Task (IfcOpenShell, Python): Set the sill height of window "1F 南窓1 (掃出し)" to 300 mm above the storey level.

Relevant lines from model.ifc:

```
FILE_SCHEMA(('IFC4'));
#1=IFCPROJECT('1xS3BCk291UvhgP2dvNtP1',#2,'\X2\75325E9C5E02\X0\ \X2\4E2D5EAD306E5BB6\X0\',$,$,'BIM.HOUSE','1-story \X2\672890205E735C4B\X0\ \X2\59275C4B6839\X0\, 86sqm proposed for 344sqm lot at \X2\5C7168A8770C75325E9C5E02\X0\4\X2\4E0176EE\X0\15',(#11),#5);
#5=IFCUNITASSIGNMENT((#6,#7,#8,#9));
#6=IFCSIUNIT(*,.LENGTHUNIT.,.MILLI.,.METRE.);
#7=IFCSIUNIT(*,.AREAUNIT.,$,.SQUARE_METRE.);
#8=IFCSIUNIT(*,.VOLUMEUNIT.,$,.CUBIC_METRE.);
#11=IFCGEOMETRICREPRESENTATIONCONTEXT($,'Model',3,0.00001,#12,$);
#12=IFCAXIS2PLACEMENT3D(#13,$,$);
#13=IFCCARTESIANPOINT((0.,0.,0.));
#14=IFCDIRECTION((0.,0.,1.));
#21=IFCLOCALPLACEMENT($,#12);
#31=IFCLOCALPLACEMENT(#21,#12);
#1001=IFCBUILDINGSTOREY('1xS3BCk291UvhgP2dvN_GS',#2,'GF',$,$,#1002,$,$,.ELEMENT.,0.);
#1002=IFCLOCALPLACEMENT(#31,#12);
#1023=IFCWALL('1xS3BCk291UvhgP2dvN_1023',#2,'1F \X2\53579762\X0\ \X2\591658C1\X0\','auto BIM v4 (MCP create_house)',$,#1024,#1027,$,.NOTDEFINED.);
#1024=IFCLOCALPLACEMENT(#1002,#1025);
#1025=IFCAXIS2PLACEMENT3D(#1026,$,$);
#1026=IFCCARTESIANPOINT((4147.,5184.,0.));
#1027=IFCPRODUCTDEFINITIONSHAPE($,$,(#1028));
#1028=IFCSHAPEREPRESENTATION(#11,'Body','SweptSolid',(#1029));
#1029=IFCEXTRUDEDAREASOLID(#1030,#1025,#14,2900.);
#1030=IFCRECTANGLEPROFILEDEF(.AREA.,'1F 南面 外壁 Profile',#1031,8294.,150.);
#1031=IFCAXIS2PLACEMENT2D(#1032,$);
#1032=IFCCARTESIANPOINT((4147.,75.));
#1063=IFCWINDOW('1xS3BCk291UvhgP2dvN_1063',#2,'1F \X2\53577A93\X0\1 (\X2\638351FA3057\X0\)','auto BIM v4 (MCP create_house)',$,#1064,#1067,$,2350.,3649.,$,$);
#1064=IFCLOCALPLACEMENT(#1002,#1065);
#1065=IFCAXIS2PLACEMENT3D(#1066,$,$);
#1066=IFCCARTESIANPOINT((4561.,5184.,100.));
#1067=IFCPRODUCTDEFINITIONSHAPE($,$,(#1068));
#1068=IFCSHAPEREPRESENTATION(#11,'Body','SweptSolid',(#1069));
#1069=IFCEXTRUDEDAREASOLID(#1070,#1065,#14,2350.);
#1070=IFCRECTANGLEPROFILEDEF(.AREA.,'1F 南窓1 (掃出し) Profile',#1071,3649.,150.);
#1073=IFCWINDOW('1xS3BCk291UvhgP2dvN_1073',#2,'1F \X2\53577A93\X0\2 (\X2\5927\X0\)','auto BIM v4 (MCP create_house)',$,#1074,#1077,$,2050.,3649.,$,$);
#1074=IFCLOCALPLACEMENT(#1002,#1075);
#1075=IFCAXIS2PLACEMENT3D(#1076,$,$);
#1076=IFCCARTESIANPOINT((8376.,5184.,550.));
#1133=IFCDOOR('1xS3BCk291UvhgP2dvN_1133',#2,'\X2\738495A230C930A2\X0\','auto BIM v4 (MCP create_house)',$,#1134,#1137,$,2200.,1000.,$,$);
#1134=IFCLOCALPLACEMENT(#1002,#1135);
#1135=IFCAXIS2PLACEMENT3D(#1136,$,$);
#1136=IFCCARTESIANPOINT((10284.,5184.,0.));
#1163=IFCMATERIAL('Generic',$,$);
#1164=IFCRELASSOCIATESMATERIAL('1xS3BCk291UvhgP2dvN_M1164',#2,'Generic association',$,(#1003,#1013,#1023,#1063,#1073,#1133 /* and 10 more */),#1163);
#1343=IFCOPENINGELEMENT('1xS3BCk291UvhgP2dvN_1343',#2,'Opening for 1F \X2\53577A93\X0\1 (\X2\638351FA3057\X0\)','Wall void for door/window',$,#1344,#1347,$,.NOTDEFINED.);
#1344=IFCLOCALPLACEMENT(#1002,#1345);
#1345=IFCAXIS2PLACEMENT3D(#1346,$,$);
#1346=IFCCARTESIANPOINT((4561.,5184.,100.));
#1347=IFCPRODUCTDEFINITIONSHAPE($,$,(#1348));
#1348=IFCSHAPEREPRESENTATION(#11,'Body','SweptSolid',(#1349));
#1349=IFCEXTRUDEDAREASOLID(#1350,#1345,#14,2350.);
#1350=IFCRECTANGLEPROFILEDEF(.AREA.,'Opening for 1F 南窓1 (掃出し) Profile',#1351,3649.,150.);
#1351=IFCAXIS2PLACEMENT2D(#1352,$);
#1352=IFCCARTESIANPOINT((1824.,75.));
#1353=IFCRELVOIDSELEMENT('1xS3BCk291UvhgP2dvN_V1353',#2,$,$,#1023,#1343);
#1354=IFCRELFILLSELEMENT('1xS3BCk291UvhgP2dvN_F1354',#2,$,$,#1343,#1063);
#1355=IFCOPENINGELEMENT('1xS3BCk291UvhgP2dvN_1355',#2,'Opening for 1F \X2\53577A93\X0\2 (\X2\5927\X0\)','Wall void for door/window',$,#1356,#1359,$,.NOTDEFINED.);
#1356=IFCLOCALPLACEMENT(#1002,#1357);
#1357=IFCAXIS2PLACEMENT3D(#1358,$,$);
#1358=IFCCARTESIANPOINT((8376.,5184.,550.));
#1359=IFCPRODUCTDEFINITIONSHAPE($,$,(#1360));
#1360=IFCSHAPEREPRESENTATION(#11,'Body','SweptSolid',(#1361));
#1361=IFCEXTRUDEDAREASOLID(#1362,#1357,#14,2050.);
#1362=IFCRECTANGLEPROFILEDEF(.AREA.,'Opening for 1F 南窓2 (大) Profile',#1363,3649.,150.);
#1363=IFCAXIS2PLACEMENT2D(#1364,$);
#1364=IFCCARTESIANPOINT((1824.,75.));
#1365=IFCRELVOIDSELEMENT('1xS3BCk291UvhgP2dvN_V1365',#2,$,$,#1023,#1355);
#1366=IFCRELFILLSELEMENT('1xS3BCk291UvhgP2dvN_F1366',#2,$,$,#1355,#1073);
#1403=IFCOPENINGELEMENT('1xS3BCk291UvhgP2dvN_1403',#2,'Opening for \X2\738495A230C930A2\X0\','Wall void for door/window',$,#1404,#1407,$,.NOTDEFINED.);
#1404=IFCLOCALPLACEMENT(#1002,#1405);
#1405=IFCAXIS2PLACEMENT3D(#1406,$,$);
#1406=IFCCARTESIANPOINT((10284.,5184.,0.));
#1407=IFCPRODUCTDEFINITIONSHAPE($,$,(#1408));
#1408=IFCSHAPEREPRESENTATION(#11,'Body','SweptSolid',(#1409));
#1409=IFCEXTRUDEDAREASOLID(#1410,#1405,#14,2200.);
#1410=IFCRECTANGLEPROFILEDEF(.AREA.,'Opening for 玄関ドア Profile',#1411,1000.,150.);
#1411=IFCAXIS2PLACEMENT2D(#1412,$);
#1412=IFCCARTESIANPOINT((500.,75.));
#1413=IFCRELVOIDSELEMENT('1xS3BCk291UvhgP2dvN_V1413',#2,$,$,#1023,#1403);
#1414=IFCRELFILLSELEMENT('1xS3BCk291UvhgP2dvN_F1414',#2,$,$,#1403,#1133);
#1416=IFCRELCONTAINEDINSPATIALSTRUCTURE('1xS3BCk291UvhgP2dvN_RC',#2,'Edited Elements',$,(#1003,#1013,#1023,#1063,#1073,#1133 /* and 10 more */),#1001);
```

```python
import numpy as np
import ifcopenshell
import ifcopenshell.api.geometry
import ifcopenshell.geom
import ifcopenshell.util.element
import ifcopenshell.util.placement
import ifcopenshell.util.shape
import ifcopenshell.util.unit

model = ifcopenshell.open("model.ifc")
unit_scale = ifcopenshell.util.unit.calculate_unit_scale(model)

window = model.by_guid("1xS3BCk291UvhgP2dvN_1063")
opening = window.FillsVoids[0].RelatingOpeningElement
storey = ifcopenshell.util.element.get_container(window, ifc_class="IfcBuildingStorey")
level = ifcopenshell.util.placement.get_local_placement(storey.ObjectPlacement)[2, 3]

# The opening's origin need not be at the sill, so measure its lowest point.
shape = ifcopenshell.geom.create_shape(ifcopenshell.geom.settings(), opening)
bottom = ifcopenshell.util.shape.get_shape_bottom_elevation(shape, shape.geometry) / unit_scale
dz = level + 0.3 / unit_scale - bottom

shift = np.array([0.0, 0.0, dz])
# The window is not placed relative to its opening, so move both.
for product in (opening, window):
    matrix = ifcopenshell.util.placement.get_local_placement(product.ObjectPlacement)
    matrix[:3, 3] += shift
    ifcopenshell.api.geometry.edit_object_placement(model, product=product, matrix=matrix, is_si=False)

print(f"moved by {dz * unit_scale:+.3f} m")

model.write("model_updated.ifc")
```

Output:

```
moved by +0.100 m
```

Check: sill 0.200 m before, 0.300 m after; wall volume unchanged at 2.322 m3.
